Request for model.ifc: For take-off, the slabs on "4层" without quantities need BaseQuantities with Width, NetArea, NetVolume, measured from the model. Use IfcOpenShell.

First a look at what the model holds.

```python
import ifcopenshell
import ifcopenshell.util.element
import ifcopenshell.util.unit

model = ifcopenshell.open("model.ifc")
print(model.schema)
for unit_type in ("LENGTHUNIT", "AREAUNIT", "VOLUMEUNIT"):
    print(unit_type, ifcopenshell.util.unit.calculate_unit_scale(model, unit_type))
storey = next(s for s in model.by_type("IfcBuildingStorey") if s.Name == "4层")
slabs = [e for e in ifcopenshell.util.element.get_decomposition(storey) if e.is_a("IfcSlab")]
for e in sorted(slabs, key=lambda e: e.id()):
    print(e.id(), e.is_a(), e.Name, list(ifcopenshell.util.element.get_psets(e, qtos_only=True)), sep=" | ")
```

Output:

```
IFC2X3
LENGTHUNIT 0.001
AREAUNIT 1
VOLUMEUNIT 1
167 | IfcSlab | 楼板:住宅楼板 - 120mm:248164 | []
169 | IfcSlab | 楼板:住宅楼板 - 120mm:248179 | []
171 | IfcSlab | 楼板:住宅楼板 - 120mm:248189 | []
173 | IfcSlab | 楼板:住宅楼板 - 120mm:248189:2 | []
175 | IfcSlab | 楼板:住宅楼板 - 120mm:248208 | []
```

```python
import ifcopenshell
import ifcopenshell.api.pset
import ifcopenshell.geom
import ifcopenshell.util.element
import ifcopenshell.util.shape
import ifcopenshell.util.unit

model = ifcopenshell.open("model.ifc")
unit_scale = ifcopenshell.util.unit.calculate_unit_scale(model)
area_scale = ifcopenshell.util.unit.calculate_unit_scale(model, "AREAUNIT")
volume_scale = ifcopenshell.util.unit.calculate_unit_scale(model, "VOLUMEUNIT")
settings = ifcopenshell.geom.settings()

storey = next(s for s in model.by_type("IfcBuildingStorey") if s.Name == "4层")
slabs = [e for e in ifcopenshell.util.element.get_decomposition(storey) if e.is_a("IfcSlab")]

for e in sorted(slabs, key=lambda e: e.id()):
    if ifcopenshell.util.element.get_psets(e, qtos_only=True, should_inherit=False):
        continue
    # Geometry comes back in metres, in the element's own axes.
    shape = ifcopenshell.geom.create_shape(settings, e)
    values = {
        "Width": ifcopenshell.util.shape.get_z(shape.geometry) / unit_scale,
        "NetArea": ifcopenshell.util.shape.get_footprint_area(shape.geometry) / area_scale,
        "NetVolume": ifcopenshell.util.shape.get_volume(shape.geometry) / volume_scale,
    }
    qto = ifcopenshell.api.pset.add_qto(model, product=e, name="BaseQuantities")
    ifcopenshell.api.pset.edit_qto(model, qto=qto, properties=values)
    print(e.id(), {k: round(v, 3) for k, v in values.items()})

model.write("model_updated.ifc")
```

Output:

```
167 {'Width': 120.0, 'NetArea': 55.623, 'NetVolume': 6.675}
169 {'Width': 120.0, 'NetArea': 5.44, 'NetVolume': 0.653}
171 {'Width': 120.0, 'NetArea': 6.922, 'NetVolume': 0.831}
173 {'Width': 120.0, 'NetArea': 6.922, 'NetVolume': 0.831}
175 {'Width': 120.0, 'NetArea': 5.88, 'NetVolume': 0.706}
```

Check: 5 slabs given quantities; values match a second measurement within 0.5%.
